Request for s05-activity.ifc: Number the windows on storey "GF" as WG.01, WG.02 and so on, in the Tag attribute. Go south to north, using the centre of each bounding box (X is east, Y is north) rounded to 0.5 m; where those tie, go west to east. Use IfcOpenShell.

First a look at what the model holds.

```python
import ifcopenshell
import ifcopenshell.util.element
import ifcopenshell.util.placement

model = ifcopenshell.open("s05-activity.ifc")
print(model.schema)
storey = next(s for s in model.by_type("IfcBuildingStorey") if s.Name == "GF")
windows = [e for e in ifcopenshell.util.element.get_decomposition(storey) if e.is_a("IfcWindow")]
for e in sorted(windows, key=lambda e: e.id()):
    origin = ifcopenshell.util.placement.get_local_placement(e.ObjectPlacement)[:3, 3]
    print(e.id(), e.Tag, e.Name, origin.round(2) + 0.0, sep=" | ")
```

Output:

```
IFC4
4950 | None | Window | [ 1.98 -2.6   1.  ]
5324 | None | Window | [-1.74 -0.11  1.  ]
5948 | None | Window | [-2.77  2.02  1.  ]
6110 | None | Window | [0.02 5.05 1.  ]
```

```python
import ifcopenshell
import ifcopenshell.geom
import ifcopenshell.util.element
import ifcopenshell.util.shape

model = ifcopenshell.open("s05-activity.ifc")
settings = ifcopenshell.geom.settings()
settings.set("use-world-coords", True)


def centre(element):
    shape = ifcopenshell.geom.create_shape(settings, element)
    return ifcopenshell.util.shape.get_bbox_centroid(shape.geometry)


storey = next(s for s in model.by_type("IfcBuildingStorey") if s.Name == "GF")
windows = [e for e in ifcopenshell.util.element.get_decomposition(storey) if e.is_a("IfcWindow")]

# Insertion points can sit at a corner or the storey origin, so sort by the geometry (in metres).
centres = {e: centre(e) for e in windows}
windows.sort(key=lambda e: (round(centres[e][1] / 0.5), centres[e][0]))

for i, e in enumerate(windows, start=1):
    number = f"WG.{i:02d}"
    e.Tag = number
    print(e.id(), number)

model.write("s05-activity_rev.ifc")
```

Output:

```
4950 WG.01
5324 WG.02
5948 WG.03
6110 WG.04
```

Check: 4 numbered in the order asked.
